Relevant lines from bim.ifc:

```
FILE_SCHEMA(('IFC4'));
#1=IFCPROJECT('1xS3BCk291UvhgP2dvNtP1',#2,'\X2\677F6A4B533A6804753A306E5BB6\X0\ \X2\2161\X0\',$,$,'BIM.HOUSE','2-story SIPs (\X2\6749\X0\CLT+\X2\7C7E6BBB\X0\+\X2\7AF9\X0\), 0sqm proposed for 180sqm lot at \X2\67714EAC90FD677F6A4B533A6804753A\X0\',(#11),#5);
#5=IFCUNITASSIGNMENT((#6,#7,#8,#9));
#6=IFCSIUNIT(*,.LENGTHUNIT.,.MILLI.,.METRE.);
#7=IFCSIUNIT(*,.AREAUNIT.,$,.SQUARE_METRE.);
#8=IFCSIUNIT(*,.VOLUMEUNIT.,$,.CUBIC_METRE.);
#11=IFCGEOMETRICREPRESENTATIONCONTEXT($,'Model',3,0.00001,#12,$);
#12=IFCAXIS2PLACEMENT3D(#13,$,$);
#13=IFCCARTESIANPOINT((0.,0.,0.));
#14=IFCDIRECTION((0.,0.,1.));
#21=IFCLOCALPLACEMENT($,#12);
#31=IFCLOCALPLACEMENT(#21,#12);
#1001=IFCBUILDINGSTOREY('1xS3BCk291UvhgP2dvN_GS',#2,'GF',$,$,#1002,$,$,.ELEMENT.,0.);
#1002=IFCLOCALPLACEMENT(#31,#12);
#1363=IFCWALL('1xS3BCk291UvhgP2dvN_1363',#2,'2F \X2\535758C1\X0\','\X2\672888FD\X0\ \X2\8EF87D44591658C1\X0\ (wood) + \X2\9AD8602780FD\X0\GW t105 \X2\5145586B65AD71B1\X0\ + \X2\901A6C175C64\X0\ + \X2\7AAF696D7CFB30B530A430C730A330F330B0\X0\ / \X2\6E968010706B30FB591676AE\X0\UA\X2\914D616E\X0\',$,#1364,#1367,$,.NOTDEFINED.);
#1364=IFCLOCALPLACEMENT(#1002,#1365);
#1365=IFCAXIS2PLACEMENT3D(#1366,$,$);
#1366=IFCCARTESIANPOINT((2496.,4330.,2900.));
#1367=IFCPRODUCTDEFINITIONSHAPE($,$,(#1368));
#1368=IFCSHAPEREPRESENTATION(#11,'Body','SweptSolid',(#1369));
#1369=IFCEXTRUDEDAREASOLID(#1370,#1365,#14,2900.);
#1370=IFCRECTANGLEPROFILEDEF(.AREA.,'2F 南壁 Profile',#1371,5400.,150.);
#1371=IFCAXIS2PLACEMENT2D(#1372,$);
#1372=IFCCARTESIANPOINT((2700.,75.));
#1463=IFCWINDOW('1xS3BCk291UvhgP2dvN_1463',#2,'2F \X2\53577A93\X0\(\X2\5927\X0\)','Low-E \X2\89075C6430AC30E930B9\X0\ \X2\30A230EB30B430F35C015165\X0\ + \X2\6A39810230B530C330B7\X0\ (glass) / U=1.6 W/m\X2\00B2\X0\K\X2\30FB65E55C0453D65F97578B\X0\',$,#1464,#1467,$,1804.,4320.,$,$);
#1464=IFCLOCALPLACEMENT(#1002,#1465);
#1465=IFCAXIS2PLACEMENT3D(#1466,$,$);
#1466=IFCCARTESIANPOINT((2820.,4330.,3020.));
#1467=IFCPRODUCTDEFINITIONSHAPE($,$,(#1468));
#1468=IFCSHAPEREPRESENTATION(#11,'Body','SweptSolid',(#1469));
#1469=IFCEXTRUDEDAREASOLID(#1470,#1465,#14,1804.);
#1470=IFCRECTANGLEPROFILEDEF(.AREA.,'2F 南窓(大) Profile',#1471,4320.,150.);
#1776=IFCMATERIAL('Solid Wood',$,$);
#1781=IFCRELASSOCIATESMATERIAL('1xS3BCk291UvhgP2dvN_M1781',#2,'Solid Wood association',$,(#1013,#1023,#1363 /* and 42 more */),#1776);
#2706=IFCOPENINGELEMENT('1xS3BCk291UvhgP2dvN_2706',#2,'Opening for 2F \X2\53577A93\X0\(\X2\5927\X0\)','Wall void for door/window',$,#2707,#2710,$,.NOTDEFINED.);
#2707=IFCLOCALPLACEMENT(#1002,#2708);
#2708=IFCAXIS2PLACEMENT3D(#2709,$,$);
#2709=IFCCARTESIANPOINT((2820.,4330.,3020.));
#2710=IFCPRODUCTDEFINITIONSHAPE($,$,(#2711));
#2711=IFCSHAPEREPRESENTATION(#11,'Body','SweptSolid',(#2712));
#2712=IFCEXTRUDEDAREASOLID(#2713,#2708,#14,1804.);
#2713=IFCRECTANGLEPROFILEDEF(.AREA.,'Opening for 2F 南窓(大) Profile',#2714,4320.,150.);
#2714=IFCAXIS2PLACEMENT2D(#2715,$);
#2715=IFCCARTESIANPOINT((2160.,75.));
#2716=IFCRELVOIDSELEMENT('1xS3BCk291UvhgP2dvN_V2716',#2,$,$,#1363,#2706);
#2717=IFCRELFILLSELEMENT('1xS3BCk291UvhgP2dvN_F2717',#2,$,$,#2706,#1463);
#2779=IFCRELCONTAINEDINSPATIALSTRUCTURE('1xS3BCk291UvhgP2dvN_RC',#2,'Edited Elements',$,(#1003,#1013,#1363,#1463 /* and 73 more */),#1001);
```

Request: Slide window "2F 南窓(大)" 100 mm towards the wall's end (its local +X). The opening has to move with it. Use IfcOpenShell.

```python
import ifcopenshell
import ifcopenshell.api.geometry
import ifcopenshell.util.placement

model = ifcopenshell.open("bim.ifc")

window = model.by_guid("1xS3BCk291UvhgP2dvN_1463")
opening = window.FillsVoids[0].RelatingOpeningElement
wall = opening.VoidsElements[0].RelatingBuildingElement

wall_matrix = ifcopenshell.util.placement.get_local_placement(wall.ObjectPlacement)
shift = wall_matrix[:3, 0] * 100.0
before = ifcopenshell.util.placement.get_local_placement(window.ObjectPlacement)[:3, 3].copy()

# The window is not placed relative to its opening, so move both.
for product in (opening, window):
    matrix = ifcopenshell.util.placement.get_local_placement(product.ObjectPlacement)
    matrix[:3, 3] += shift
    ifcopenshell.api.geometry.edit_object_placement(model, product=product, matrix=matrix, is_si=False)

after = ifcopenshell.util.placement.get_local_placement(window.ObjectPlacement)[:3, 3]
print("window moved by", (after - before).round(3) + 0.0)

model.write("bim_updated.ifc")
```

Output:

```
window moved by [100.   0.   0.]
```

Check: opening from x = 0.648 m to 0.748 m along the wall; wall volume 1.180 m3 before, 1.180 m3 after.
